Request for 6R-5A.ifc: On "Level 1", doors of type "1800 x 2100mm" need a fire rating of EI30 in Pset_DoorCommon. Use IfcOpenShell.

First a look at what the model holds.

```python
import ifcopenshell
import ifcopenshell.util.element

model = ifcopenshell.open("6R-5A.ifc")
print(model.schema)
storey = next(s for s in model.by_type("IfcBuildingStorey") if s.Name == "Level 1")
doors = [e for e in ifcopenshell.util.element.get_decomposition(storey) if e.is_a("IfcDoor")]
seen = {}
for e in doors:
    element_type = ifcopenshell.util.element.get_type(e)
    key = (element_type.Name if element_type != e and element_type else None, ifcopenshell.util.element.get_pset(e, "Pset_DoorCommon", "FireRating"))
    seen[key] = seen.get(key, 0) + 1
for (name, value), count in sorted(seen.items(), key=str):
    print(count, "x", name, "|", value)
```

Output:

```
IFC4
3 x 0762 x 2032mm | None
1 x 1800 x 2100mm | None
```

```python
import ifcopenshell
import ifcopenshell.api.pset
import ifcopenshell.util.element

model = ifcopenshell.open("6R-5A.ifc")

storey = next(s for s in model.by_type("IfcBuildingStorey") if s.Name == "Level 1")
doors = [e for e in ifcopenshell.util.element.get_decomposition(storey) if e.is_a("IfcDoor")]

count = 0
for e in doors:
    element_type = ifcopenshell.util.element.get_type(e)
    if element_type in (None, e) or element_type.Name != "1800 x 2100mm":
        continue
    # add_pset returns the element's existing set when there is one.
    pset = ifcopenshell.api.pset.add_pset(model, product=e, name="Pset_DoorCommon")
    ifcopenshell.api.pset.edit_pset(model, pset=pset, properties={"FireRating": "EI30"})
    count += 1

print(count, "doors updated")

model.write("6R-5A_edited.ifc")
```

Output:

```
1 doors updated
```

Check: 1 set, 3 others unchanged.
